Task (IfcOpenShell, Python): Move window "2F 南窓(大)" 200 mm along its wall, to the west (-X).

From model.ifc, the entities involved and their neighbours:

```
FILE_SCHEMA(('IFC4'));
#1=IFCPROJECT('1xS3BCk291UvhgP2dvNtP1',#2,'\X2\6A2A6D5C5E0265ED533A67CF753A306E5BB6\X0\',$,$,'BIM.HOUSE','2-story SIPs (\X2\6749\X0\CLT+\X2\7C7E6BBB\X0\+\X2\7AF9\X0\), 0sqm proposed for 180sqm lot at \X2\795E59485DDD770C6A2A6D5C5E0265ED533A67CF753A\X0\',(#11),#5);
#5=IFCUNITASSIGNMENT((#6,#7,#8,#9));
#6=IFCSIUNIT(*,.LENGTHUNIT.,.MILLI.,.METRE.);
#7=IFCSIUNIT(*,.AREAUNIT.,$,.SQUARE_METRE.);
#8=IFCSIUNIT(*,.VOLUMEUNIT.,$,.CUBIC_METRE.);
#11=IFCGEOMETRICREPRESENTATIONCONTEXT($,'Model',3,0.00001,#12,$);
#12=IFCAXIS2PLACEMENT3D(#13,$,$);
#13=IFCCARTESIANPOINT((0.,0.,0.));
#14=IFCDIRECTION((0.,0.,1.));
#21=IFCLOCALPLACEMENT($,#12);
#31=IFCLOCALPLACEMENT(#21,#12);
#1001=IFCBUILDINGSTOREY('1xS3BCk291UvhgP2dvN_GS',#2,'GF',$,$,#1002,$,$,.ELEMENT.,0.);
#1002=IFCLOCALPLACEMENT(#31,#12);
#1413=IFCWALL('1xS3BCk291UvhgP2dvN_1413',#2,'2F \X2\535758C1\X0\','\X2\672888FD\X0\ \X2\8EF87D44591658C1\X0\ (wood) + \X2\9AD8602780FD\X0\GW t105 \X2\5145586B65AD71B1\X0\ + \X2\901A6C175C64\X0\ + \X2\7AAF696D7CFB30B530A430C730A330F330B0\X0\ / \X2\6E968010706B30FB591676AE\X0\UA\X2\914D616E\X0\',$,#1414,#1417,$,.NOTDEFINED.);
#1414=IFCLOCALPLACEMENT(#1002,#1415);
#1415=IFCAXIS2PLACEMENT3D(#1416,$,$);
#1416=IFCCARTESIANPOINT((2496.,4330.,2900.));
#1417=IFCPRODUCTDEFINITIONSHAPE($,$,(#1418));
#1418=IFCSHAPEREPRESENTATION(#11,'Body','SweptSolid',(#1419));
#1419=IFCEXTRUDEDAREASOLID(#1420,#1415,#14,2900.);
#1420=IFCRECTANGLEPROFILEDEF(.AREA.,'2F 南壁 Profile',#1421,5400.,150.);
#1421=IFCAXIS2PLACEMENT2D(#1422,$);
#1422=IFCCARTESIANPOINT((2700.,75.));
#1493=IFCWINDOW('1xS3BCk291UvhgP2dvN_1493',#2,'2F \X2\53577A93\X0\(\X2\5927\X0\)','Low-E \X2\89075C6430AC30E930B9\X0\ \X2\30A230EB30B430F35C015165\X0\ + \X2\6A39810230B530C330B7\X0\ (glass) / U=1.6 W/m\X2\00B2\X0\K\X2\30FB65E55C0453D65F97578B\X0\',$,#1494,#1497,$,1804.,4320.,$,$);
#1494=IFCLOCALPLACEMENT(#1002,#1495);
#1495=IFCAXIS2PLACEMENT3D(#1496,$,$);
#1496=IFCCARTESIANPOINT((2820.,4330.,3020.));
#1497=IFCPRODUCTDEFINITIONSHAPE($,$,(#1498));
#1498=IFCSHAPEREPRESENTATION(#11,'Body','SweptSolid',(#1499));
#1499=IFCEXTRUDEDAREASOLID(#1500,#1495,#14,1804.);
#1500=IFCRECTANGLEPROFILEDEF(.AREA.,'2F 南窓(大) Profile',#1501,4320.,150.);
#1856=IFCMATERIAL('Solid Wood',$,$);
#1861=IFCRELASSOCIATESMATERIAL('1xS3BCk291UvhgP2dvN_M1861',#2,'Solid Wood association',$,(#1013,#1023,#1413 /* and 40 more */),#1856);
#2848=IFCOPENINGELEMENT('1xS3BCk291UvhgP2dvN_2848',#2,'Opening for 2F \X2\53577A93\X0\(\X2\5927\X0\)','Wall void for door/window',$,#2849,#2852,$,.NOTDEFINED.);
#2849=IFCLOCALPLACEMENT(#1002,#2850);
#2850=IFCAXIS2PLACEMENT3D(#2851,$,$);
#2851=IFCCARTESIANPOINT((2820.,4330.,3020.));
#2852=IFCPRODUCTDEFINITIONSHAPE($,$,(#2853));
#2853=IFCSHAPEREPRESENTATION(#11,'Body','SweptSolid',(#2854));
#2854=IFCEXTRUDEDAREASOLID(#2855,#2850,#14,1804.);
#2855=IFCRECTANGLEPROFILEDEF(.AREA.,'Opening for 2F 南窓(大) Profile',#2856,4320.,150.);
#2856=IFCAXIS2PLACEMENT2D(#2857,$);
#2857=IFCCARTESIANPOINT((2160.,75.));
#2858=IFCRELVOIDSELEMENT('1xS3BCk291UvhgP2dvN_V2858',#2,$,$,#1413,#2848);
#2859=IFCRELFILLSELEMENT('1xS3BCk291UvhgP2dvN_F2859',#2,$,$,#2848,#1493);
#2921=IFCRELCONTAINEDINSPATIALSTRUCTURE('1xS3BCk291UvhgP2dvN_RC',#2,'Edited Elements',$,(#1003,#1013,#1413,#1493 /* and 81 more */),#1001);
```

```python
import ifcopenshell
import ifcopenshell.api.geometry
import ifcopenshell.util.placement
import ifcopenshell.util.unit

model = ifcopenshell.open("model.ifc")
unit_scale = ifcopenshell.util.unit.calculate_unit_scale(model)

window = model.by_guid("1xS3BCk291UvhgP2dvN_1493")
opening = window.FillsVoids[0].RelatingOpeningElement
wall = opening.VoidsElements[0].RelatingBuildingElement

wall_matrix = ifcopenshell.util.placement.get_local_placement(wall.ObjectPlacement)
shift = wall_matrix[:3, 0] * -0.2 / unit_scale
before = ifcopenshell.util.placement.get_local_placement(window.ObjectPlacement)[:3, 3].copy()

# The window is not placed relative to its opening, so move both.
for product in (opening, window):
    matrix = ifcopenshell.util.placement.get_local_placement(product.ObjectPlacement)
    matrix[:3, 3] += shift
    ifcopenshell.api.geometry.edit_object_placement(model, product=product, matrix=matrix, is_si=False)

after = ifcopenshell.util.placement.get_local_placement(window.ObjectPlacement)[:3, 3]
print("window moved by", (after - before).round(3) + 0.0)

model.write("model-out.ifc")
```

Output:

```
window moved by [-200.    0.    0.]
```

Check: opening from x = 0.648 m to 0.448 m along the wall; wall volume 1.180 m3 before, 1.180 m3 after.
